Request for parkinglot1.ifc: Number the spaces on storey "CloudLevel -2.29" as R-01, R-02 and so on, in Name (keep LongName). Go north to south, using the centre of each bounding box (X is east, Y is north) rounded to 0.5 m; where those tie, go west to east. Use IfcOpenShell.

First a look at what the model holds.

```python
import ifcopenshell
import ifcopenshell.util.element
import ifcopenshell.util.placement

model = ifcopenshell.open("parkinglot1.ifc")
print(model.schema)
storey = next(s for s in model.by_type("IfcBuildingStorey") if s.Name == "CloudLevel -2.29")
spaces = [e for e in ifcopenshell.util.element.get_decomposition(storey) if e.is_a("IfcSpace")]
for e in sorted(spaces, key=lambda e: e.id()):
    origin = ifcopenshell.util.placement.get_local_placement(e.ObjectPlacement)[:3, 3]
    print(e.id(), e.Name, e.LongName, origin.round(2) + 0.0, sep=" | ")
```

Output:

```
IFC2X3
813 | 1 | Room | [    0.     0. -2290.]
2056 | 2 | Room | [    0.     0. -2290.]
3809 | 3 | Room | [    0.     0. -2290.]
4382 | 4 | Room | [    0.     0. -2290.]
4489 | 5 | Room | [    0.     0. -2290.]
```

```python
import ifcopenshell
import ifcopenshell.geom
import ifcopenshell.util.element
import ifcopenshell.util.shape

model = ifcopenshell.open("parkinglot1.ifc")
settings = ifcopenshell.geom.settings()
settings.set("use-world-coords", True)


def centre(element):
    shape = ifcopenshell.geom.create_shape(settings, element)
    return ifcopenshell.util.shape.get_bbox_centroid(shape.geometry)


storey = next(s for s in model.by_type("IfcBuildingStorey") if s.Name == "CloudLevel -2.29")
spaces = [e for e in ifcopenshell.util.element.get_decomposition(storey) if e.is_a("IfcSpace")]

# Insertion points can sit at a corner or the storey origin, so sort by the geometry (in metres).
centres = {e: centre(e) for e in spaces}
spaces.sort(key=lambda e: (-round(centres[e][1] / 0.5), centres[e][0]))

for i, e in enumerate(spaces, start=1):
    number = f"R-{i:02d}"
    e.Name = number
    print(e.id(), number)

model.write("parkinglot1_updated.ifc")
```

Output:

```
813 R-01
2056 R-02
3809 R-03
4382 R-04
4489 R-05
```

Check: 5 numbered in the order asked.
